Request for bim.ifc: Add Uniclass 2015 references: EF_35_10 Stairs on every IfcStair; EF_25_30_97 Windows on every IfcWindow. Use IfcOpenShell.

First a look at what the model holds.

```python
import ifcopenshell

model = ifcopenshell.open("bim.ifc")
print(model.schema)
print("classifications:", [c.Name for c in model.by_type("IfcClassification")])
for ifc_class in ("IfcDoor", "IfcRoof", "IfcStair", "IfcWall", "IfcWindow"):
    print(ifc_class, len(model.by_type(ifc_class)))
```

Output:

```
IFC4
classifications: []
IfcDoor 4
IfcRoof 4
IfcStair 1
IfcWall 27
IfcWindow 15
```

```python
import ifcopenshell
import ifcopenshell.api.classification

model = ifcopenshell.open("bim.ifc")

system = ifcopenshell.api.classification.add_classification(model, classification="Uniclass 2015")

codes = {
    "IfcStair": ("EF_35_10", "Stairs"),
    "IfcWindow": ("EF_25_30_97", "Windows"),
}
for ifc_class, (code, name) in codes.items():
    products = model.by_type(ifc_class)
    ifcopenshell.api.classification.add_reference(
        model, products=products, classification=system, identification=code, name=name
    )
    print(code, len(products))

model.write("bim_edited.ifc")
```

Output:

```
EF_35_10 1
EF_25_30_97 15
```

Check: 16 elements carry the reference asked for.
